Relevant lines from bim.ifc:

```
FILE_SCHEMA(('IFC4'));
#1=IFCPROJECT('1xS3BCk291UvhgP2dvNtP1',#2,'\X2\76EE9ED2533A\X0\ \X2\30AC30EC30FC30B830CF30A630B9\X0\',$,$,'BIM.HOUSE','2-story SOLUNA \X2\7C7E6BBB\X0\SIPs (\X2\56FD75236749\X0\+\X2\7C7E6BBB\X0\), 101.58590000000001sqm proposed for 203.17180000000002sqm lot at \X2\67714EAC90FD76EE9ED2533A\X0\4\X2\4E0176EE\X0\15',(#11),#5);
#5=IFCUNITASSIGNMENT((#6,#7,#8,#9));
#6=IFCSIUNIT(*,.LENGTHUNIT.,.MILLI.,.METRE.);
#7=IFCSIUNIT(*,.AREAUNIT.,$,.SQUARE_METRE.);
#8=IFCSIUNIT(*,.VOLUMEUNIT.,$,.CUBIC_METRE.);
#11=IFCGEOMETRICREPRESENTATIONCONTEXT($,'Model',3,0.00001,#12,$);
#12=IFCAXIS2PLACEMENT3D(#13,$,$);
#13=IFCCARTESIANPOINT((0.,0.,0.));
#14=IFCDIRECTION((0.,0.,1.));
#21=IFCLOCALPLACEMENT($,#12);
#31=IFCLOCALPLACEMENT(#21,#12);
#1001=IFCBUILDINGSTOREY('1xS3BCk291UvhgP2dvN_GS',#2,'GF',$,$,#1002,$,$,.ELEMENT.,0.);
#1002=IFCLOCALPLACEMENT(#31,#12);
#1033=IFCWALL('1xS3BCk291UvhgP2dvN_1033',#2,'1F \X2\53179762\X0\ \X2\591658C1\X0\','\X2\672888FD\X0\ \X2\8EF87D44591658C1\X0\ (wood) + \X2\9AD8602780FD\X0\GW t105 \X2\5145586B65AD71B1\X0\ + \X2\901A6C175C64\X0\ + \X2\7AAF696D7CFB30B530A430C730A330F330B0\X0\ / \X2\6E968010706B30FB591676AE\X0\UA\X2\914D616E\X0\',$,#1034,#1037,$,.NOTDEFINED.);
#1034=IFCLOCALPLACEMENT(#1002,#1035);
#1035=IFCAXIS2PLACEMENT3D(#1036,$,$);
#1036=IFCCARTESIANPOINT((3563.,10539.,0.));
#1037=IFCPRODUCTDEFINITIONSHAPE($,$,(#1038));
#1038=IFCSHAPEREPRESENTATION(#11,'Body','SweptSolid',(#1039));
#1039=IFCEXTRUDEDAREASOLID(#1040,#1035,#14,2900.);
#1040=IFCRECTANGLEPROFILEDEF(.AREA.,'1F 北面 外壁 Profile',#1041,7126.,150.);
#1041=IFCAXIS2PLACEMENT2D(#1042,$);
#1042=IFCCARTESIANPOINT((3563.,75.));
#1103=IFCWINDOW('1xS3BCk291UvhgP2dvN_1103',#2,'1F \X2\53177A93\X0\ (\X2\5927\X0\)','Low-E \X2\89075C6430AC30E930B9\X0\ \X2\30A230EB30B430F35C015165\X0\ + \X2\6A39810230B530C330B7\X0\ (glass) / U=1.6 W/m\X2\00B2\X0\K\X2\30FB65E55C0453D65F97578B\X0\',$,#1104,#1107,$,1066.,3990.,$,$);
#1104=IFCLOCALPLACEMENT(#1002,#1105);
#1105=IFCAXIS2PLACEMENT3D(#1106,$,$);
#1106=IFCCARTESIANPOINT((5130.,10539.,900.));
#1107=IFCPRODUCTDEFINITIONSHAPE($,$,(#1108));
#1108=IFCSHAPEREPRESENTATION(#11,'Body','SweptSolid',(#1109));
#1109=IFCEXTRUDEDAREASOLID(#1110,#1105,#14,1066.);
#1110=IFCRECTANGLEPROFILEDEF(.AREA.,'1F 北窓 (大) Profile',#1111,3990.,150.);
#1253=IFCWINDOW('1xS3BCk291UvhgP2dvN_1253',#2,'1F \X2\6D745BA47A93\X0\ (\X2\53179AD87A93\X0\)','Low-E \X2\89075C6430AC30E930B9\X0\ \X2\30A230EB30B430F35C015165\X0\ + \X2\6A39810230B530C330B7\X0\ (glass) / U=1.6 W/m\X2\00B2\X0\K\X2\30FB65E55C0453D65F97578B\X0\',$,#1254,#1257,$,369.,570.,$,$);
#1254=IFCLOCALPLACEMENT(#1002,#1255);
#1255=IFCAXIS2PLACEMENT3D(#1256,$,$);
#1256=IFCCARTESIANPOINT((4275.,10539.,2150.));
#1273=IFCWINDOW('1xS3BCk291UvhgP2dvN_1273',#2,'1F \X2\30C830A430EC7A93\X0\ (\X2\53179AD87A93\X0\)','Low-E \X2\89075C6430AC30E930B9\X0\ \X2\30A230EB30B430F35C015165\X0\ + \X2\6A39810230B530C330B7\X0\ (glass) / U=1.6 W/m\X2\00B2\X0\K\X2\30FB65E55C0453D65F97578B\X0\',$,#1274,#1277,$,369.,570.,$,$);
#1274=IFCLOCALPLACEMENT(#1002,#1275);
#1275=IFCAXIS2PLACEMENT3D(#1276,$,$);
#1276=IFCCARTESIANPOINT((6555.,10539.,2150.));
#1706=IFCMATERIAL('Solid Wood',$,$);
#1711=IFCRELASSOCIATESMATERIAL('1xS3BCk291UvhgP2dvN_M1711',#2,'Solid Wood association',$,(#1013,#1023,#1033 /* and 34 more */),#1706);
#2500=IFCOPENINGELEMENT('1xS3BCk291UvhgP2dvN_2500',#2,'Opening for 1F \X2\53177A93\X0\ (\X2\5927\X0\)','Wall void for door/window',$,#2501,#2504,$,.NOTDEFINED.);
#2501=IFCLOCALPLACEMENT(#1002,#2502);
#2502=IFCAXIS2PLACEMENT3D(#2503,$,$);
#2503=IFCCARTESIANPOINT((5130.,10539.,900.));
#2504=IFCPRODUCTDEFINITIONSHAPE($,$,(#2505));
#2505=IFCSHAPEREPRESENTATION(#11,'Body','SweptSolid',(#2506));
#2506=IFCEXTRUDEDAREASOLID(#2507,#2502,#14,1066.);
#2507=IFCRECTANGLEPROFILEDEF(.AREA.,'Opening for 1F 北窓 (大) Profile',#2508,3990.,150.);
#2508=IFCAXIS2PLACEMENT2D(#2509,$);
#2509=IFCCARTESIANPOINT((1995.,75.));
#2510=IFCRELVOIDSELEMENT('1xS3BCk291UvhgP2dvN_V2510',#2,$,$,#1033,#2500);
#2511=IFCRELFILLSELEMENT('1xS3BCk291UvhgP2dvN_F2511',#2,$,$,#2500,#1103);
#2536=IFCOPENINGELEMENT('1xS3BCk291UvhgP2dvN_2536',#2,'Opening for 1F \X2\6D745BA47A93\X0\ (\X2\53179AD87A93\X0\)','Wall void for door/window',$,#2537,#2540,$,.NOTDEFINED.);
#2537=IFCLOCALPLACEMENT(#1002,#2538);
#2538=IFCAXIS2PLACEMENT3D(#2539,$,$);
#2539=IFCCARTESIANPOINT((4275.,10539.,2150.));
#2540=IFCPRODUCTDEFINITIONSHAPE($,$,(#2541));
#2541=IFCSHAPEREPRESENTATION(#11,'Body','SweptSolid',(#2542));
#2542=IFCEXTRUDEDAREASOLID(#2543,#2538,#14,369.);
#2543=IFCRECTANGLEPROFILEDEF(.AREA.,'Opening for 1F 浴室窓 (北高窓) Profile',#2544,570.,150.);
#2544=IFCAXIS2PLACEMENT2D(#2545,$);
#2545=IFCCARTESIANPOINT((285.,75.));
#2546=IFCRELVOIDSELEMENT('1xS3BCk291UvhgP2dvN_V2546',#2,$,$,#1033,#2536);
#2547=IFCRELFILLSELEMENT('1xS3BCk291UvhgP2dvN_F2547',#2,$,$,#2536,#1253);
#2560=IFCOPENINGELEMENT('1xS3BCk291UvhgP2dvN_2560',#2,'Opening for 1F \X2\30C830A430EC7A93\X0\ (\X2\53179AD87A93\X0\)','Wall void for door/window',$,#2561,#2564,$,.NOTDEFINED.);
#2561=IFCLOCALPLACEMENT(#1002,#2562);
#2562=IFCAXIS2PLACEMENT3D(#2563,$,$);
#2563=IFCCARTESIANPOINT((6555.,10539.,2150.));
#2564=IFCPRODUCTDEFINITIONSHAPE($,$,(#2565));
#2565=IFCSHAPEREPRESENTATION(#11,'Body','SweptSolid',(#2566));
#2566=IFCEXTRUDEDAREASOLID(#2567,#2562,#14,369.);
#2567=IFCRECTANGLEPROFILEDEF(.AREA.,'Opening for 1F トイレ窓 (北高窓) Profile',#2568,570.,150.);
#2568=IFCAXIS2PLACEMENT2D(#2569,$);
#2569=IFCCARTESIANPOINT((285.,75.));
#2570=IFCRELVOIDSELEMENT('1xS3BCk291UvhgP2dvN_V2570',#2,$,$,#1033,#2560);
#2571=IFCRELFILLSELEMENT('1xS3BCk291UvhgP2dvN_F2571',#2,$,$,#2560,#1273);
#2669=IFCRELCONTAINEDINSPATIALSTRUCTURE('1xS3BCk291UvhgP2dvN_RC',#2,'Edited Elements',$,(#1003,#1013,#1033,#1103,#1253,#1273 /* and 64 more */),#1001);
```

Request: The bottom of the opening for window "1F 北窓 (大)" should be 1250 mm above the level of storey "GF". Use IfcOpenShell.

```python
import numpy as np
import ifcopenshell
import ifcopenshell.api.geometry
import ifcopenshell.geom
import ifcopenshell.util.element
import ifcopenshell.util.placement
import ifcopenshell.util.shape
import ifcopenshell.util.unit

model = ifcopenshell.open("bim.ifc")
unit_scale = ifcopenshell.util.unit.calculate_unit_scale(model)

window = model.by_guid("1xS3BCk291UvhgP2dvN_1103")
opening = window.FillsVoids[0].RelatingOpeningElement
storey = ifcopenshell.util.element.get_container(window, ifc_class="IfcBuildingStorey")
level = ifcopenshell.util.placement.get_local_placement(storey.ObjectPlacement)[2, 3]

# The opening's origin need not be at the sill, so measure its lowest point.
shape = ifcopenshell.geom.create_shape(ifcopenshell.geom.settings(), opening)
bottom = ifcopenshell.util.shape.get_shape_bottom_elevation(shape, shape.geometry) / unit_scale
dz = level + 1.25 / unit_scale - bottom

shift = np.array([0.0, 0.0, dz])
# The window is not placed relative to its opening, so move both.
for product in (opening, window):
    matrix = ifcopenshell.util.placement.get_local_placement(product.ObjectPlacement)
    matrix[:3, 3] += shift
    ifcopenshell.api.geometry.edit_object_placement(model, product=product, matrix=matrix, is_si=False)

print(f"moved by {dz * unit_scale:+.3f} m")

model.write("bim_updated.ifc")
```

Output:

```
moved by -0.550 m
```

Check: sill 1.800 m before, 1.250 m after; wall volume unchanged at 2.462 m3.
